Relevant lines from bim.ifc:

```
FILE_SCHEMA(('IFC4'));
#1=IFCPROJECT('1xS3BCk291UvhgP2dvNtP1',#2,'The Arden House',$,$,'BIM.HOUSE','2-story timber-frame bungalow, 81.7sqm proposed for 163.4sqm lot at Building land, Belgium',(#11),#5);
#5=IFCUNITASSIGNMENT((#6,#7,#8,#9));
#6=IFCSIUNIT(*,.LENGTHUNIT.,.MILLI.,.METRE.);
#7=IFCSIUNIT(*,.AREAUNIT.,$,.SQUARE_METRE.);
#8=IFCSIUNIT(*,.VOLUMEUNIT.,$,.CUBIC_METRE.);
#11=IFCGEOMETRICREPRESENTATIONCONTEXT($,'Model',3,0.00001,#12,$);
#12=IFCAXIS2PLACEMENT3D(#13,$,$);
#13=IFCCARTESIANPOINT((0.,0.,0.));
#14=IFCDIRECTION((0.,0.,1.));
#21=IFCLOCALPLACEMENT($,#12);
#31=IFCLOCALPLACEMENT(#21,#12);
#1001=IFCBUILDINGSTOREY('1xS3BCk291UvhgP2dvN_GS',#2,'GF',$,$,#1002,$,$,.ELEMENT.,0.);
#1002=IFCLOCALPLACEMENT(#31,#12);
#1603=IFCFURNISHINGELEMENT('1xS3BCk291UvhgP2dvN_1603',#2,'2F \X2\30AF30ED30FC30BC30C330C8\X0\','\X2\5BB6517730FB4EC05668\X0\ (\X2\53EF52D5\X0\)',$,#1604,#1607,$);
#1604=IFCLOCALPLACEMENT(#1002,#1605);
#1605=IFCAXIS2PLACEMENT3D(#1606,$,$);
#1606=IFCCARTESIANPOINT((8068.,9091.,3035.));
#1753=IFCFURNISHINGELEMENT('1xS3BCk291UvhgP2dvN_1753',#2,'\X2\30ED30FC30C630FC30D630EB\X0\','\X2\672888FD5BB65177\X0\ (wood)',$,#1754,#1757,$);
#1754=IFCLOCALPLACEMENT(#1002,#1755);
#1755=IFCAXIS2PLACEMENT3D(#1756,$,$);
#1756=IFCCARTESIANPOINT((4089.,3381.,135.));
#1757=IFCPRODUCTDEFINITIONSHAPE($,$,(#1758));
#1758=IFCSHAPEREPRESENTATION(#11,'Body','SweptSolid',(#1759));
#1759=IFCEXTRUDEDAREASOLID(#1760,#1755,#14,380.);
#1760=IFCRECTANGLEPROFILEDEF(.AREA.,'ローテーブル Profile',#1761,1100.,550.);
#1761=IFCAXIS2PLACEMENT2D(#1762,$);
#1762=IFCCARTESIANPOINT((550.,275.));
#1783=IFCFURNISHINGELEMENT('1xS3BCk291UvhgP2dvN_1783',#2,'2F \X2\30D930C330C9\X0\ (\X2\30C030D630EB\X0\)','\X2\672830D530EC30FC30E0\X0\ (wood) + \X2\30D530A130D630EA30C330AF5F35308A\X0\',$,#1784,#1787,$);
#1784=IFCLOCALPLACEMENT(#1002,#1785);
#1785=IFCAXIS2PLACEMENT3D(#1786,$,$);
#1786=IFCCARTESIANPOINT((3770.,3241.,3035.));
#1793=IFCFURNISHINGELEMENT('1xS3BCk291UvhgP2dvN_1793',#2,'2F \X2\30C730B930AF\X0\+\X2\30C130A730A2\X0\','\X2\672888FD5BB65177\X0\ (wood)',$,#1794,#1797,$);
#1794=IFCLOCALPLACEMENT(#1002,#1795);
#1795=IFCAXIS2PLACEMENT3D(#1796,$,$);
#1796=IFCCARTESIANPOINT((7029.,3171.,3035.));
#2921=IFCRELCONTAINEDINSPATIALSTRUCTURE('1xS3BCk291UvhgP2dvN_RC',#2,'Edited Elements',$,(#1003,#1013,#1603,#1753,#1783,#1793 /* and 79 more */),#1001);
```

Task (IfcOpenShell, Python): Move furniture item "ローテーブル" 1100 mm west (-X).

```python
import ifcopenshell
import ifcopenshell.api.geometry
import ifcopenshell.util.placement

model = ifcopenshell.open("bim.ifc")

item = model.by_id(1753)
matrix = ifcopenshell.util.placement.get_local_placement(item.ObjectPlacement)
matrix[0, 3] -= 1100.0
ifcopenshell.api.geometry.edit_object_placement(model, product=item, matrix=matrix, is_si=False)

print(ifcopenshell.util.placement.get_local_placement(item.ObjectPlacement).round(3) + 0.0)

model.write("bim_updated.ifc")
```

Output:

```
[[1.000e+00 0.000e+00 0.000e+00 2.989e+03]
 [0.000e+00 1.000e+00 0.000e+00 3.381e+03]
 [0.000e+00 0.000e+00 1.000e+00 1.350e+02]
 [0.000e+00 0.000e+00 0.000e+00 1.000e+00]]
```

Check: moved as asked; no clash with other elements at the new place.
